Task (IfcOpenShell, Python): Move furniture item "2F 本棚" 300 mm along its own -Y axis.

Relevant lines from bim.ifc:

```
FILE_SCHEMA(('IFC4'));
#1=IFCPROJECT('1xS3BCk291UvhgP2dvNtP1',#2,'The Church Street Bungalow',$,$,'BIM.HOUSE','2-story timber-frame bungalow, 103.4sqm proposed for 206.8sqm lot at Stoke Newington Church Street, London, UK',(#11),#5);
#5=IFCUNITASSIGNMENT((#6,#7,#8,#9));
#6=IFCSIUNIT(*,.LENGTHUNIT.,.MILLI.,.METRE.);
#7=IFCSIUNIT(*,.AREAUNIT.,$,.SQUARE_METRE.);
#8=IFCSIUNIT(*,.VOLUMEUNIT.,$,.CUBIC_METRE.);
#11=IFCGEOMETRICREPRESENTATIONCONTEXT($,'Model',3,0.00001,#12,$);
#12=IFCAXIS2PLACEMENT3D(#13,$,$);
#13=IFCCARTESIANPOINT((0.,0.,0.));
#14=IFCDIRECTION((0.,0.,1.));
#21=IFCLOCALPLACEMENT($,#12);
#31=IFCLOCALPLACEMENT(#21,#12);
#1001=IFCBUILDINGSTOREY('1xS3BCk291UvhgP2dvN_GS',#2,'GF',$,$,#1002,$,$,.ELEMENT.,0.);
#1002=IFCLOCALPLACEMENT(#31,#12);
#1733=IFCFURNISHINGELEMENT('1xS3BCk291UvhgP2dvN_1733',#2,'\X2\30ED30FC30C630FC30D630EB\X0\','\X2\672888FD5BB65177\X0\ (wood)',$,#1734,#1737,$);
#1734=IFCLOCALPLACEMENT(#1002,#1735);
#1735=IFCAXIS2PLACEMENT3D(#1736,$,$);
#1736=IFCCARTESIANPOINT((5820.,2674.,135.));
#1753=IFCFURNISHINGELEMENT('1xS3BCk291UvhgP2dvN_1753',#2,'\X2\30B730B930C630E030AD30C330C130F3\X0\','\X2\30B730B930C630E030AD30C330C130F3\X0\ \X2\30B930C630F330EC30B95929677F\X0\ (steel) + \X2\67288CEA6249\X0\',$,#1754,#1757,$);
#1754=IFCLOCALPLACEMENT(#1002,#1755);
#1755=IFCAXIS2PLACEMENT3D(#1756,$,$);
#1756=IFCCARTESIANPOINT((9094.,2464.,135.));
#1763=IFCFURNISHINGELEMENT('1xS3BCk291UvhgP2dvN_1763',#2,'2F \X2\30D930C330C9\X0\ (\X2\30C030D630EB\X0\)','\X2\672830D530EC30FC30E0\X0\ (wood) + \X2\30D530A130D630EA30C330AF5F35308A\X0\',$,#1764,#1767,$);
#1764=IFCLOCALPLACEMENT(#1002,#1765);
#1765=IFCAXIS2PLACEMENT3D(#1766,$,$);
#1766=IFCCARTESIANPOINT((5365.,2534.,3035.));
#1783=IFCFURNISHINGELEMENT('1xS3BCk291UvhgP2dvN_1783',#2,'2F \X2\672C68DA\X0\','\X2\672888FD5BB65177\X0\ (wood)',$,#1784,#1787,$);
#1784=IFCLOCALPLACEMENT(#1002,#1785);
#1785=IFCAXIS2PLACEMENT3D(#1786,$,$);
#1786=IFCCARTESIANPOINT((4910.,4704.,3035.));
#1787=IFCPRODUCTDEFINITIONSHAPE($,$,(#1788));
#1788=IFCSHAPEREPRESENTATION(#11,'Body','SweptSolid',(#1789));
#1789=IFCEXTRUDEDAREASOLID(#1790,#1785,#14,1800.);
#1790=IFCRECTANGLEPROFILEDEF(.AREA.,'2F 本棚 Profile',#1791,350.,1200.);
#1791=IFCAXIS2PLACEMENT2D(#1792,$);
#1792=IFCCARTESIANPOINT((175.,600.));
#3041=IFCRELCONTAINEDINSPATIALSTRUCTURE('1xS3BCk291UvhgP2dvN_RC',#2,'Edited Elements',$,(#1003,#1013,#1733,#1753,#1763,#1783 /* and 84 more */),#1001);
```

```python
import ifcopenshell
import ifcopenshell.api.geometry
import ifcopenshell.util.placement
import ifcopenshell.util.unit

model = ifcopenshell.open("bim.ifc")
unit_scale = ifcopenshell.util.unit.calculate_unit_scale(model)

item = model.by_guid("1xS3BCk291UvhgP2dvN_1783")
matrix = ifcopenshell.util.placement.get_local_placement(item.ObjectPlacement)
matrix[:3, 3] -= matrix[:3, 1] * 0.3 / unit_scale
ifcopenshell.api.geometry.edit_object_placement(model, product=item, matrix=matrix, is_si=False)

print(ifcopenshell.util.placement.get_local_placement(item.ObjectPlacement).round(3) + 0.0)

model.write("bim-out.ifc")
```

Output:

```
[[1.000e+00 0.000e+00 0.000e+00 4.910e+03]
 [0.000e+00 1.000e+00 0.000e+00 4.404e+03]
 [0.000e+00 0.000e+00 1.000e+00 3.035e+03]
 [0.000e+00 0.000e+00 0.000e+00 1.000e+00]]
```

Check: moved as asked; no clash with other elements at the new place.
